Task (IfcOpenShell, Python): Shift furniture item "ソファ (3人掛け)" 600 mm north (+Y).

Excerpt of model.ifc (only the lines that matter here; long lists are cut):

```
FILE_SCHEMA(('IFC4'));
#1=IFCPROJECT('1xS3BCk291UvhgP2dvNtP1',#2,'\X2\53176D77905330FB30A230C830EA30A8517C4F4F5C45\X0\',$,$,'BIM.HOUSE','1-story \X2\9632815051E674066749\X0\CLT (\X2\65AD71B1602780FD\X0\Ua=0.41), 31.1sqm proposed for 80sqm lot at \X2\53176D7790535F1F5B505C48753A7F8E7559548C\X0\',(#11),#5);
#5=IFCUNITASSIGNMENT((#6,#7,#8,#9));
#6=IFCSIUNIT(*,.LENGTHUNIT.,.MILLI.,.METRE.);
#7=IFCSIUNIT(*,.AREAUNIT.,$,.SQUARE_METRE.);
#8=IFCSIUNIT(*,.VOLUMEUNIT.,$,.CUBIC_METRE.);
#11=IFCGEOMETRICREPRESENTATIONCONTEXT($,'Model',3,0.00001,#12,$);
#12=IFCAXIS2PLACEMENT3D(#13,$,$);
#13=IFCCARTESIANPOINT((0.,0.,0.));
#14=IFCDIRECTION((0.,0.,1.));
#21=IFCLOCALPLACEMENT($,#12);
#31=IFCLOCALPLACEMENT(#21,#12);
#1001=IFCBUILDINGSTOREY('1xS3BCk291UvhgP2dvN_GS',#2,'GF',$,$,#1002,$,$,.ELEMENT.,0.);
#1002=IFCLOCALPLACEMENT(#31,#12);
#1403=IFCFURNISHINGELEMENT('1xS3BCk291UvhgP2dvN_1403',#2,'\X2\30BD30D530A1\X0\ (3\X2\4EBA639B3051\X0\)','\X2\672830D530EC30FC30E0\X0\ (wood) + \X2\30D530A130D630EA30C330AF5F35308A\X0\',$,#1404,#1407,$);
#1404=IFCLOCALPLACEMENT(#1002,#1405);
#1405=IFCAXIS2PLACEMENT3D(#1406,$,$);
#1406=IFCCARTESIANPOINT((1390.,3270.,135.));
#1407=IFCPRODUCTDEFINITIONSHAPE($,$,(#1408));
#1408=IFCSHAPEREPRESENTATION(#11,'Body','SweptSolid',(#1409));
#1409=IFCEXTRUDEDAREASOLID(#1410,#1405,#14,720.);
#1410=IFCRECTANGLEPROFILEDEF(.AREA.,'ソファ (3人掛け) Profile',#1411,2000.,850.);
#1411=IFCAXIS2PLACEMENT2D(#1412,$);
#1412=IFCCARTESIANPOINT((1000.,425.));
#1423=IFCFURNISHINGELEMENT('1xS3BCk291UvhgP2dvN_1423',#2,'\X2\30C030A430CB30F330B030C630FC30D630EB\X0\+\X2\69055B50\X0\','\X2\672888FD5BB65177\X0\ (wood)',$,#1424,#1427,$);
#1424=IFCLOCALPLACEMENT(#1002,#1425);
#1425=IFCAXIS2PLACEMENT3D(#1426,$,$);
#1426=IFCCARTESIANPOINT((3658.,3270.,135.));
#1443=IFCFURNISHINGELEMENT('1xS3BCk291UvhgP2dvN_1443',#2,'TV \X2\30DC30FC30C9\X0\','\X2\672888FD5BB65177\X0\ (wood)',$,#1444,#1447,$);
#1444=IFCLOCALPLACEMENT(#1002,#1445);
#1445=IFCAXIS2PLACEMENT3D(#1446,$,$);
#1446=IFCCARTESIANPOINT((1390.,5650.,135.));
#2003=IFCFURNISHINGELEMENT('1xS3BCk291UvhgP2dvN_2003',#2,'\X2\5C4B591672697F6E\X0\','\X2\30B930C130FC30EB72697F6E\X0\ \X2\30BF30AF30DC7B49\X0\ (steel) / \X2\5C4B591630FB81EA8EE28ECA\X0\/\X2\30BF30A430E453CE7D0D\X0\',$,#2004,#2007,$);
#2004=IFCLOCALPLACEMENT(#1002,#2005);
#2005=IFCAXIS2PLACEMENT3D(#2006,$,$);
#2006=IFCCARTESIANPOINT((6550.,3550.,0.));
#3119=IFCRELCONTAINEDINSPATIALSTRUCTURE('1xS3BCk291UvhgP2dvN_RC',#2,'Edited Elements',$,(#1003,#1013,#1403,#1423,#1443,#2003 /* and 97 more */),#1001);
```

```python
import ifcopenshell
import ifcopenshell.api.geometry
import ifcopenshell.util.placement
import ifcopenshell.util.unit

model = ifcopenshell.open("model.ifc")
unit_scale = ifcopenshell.util.unit.calculate_unit_scale(model)

item = model.by_guid("1xS3BCk291UvhgP2dvN_1403")
matrix = ifcopenshell.util.placement.get_local_placement(item.ObjectPlacement)
matrix[1, 3] += 0.6 / unit_scale
ifcopenshell.api.geometry.edit_object_placement(model, product=item, matrix=matrix, is_si=False)

print(ifcopenshell.util.placement.get_local_placement(item.ObjectPlacement).round(3) + 0.0)

model.write("model_rev.ifc")
```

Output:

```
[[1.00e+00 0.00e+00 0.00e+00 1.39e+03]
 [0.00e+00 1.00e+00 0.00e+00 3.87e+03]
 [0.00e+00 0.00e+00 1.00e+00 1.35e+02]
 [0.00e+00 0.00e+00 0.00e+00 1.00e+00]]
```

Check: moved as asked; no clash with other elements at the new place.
